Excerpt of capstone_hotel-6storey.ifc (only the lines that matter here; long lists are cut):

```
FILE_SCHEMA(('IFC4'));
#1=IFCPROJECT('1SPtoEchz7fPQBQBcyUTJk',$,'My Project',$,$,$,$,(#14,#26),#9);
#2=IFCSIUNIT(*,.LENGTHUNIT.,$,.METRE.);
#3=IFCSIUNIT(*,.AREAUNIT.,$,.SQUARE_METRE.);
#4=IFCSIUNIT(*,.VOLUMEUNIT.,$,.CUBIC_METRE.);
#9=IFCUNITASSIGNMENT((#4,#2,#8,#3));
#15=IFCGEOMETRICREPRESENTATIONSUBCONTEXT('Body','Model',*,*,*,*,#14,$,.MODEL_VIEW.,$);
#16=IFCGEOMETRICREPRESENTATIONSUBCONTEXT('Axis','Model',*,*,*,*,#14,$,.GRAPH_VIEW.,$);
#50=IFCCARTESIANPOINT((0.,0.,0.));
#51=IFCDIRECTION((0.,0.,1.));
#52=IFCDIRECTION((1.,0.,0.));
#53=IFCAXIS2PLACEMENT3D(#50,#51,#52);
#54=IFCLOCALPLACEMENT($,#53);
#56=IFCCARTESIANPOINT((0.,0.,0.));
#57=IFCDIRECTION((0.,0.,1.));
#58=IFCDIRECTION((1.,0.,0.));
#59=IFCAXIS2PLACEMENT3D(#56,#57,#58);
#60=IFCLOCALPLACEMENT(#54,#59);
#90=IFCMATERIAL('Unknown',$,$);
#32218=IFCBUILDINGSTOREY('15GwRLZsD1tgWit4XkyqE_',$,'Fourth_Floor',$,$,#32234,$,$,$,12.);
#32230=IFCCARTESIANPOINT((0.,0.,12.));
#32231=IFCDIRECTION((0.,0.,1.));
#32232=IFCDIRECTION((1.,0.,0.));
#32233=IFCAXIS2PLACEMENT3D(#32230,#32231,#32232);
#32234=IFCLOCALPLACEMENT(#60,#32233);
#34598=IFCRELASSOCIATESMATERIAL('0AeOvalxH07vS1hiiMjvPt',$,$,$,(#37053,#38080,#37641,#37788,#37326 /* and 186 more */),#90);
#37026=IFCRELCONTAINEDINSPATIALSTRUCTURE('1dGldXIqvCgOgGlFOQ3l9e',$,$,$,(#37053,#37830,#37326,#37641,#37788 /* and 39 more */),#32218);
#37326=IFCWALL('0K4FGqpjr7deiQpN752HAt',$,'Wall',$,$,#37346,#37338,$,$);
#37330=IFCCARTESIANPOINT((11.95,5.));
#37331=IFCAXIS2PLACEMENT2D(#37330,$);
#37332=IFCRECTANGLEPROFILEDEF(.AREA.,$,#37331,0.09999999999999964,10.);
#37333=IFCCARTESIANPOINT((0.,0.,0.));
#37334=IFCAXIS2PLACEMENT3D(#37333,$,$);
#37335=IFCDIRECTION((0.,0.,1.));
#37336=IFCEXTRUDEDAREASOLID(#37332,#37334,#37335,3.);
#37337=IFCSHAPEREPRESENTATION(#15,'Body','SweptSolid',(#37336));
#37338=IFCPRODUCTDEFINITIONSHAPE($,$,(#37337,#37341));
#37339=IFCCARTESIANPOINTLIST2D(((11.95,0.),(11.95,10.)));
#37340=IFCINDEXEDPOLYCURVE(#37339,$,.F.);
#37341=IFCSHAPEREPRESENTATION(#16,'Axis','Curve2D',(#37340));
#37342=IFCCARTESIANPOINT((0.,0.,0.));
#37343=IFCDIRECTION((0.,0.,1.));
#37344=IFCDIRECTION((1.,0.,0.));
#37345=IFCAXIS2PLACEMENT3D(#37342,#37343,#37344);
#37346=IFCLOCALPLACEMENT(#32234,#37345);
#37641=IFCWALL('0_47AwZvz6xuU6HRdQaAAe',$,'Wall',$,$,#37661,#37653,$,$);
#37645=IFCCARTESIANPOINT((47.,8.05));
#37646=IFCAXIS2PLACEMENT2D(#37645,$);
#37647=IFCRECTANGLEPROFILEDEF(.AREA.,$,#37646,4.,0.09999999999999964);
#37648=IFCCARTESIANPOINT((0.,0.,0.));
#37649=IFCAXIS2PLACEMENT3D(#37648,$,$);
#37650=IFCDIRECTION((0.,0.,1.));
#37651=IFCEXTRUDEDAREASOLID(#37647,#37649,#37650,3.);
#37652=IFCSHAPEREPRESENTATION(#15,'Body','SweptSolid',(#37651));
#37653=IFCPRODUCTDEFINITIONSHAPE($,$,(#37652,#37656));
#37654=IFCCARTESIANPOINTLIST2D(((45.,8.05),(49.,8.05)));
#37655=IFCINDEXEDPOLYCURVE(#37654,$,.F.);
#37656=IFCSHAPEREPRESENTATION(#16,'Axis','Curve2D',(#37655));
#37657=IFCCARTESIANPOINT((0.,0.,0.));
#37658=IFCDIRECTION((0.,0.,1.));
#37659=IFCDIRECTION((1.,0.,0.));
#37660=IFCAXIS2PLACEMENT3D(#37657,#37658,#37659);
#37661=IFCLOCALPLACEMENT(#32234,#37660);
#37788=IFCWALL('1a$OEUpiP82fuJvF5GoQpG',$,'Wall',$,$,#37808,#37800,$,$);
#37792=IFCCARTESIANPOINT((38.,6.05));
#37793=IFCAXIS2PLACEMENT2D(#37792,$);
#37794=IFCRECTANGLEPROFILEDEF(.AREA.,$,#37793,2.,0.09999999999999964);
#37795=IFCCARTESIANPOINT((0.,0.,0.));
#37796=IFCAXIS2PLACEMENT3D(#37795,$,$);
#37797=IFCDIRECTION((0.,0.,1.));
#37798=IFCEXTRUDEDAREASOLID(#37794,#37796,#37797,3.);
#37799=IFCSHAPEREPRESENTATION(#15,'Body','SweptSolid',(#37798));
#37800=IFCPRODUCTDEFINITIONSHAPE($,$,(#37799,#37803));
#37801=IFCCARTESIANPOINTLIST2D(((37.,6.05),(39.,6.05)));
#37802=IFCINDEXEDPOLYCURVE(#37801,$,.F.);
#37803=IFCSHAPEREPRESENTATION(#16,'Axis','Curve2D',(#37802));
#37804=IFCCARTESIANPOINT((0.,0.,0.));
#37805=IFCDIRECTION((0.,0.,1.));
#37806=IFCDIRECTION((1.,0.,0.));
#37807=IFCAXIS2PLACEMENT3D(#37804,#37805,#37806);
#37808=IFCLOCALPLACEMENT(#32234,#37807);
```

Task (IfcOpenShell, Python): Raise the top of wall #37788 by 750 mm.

```python
import ifcopenshell
import ifcopenshell.geom
import ifcopenshell.util.representation
import ifcopenshell.util.shape
import ifcopenshell.util.unit

model = ifcopenshell.open("capstone_hotel-6storey.ifc")
unit_scale = ifcopenshell.util.unit.calculate_unit_scale(model)
settings = ifcopenshell.geom.settings()


def volume(element):
    """Net volume in cubic metres, openings subtracted."""
    shape = ifcopenshell.geom.create_shape(settings, element)
    return ifcopenshell.util.shape.get_volume(shape.geometry)


wall = model.by_guid("1a$OEUpiP82fuJvF5GoQpG")
before = volume(wall)

body = ifcopenshell.util.representation.get_representation(wall, "Model", "Body")
solid = body.Items[0]
old_height = solid.Depth
solid.Depth += 0.75 / unit_scale
after = volume(wall)

print(f"height {old_height:g} -> {solid.Depth:g}, volume {before:.3f} -> {after:.3f} m3")

model.write("capstone_hotel-6storey-out.ifc")
```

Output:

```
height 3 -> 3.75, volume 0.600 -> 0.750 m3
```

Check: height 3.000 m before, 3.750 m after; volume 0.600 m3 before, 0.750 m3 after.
